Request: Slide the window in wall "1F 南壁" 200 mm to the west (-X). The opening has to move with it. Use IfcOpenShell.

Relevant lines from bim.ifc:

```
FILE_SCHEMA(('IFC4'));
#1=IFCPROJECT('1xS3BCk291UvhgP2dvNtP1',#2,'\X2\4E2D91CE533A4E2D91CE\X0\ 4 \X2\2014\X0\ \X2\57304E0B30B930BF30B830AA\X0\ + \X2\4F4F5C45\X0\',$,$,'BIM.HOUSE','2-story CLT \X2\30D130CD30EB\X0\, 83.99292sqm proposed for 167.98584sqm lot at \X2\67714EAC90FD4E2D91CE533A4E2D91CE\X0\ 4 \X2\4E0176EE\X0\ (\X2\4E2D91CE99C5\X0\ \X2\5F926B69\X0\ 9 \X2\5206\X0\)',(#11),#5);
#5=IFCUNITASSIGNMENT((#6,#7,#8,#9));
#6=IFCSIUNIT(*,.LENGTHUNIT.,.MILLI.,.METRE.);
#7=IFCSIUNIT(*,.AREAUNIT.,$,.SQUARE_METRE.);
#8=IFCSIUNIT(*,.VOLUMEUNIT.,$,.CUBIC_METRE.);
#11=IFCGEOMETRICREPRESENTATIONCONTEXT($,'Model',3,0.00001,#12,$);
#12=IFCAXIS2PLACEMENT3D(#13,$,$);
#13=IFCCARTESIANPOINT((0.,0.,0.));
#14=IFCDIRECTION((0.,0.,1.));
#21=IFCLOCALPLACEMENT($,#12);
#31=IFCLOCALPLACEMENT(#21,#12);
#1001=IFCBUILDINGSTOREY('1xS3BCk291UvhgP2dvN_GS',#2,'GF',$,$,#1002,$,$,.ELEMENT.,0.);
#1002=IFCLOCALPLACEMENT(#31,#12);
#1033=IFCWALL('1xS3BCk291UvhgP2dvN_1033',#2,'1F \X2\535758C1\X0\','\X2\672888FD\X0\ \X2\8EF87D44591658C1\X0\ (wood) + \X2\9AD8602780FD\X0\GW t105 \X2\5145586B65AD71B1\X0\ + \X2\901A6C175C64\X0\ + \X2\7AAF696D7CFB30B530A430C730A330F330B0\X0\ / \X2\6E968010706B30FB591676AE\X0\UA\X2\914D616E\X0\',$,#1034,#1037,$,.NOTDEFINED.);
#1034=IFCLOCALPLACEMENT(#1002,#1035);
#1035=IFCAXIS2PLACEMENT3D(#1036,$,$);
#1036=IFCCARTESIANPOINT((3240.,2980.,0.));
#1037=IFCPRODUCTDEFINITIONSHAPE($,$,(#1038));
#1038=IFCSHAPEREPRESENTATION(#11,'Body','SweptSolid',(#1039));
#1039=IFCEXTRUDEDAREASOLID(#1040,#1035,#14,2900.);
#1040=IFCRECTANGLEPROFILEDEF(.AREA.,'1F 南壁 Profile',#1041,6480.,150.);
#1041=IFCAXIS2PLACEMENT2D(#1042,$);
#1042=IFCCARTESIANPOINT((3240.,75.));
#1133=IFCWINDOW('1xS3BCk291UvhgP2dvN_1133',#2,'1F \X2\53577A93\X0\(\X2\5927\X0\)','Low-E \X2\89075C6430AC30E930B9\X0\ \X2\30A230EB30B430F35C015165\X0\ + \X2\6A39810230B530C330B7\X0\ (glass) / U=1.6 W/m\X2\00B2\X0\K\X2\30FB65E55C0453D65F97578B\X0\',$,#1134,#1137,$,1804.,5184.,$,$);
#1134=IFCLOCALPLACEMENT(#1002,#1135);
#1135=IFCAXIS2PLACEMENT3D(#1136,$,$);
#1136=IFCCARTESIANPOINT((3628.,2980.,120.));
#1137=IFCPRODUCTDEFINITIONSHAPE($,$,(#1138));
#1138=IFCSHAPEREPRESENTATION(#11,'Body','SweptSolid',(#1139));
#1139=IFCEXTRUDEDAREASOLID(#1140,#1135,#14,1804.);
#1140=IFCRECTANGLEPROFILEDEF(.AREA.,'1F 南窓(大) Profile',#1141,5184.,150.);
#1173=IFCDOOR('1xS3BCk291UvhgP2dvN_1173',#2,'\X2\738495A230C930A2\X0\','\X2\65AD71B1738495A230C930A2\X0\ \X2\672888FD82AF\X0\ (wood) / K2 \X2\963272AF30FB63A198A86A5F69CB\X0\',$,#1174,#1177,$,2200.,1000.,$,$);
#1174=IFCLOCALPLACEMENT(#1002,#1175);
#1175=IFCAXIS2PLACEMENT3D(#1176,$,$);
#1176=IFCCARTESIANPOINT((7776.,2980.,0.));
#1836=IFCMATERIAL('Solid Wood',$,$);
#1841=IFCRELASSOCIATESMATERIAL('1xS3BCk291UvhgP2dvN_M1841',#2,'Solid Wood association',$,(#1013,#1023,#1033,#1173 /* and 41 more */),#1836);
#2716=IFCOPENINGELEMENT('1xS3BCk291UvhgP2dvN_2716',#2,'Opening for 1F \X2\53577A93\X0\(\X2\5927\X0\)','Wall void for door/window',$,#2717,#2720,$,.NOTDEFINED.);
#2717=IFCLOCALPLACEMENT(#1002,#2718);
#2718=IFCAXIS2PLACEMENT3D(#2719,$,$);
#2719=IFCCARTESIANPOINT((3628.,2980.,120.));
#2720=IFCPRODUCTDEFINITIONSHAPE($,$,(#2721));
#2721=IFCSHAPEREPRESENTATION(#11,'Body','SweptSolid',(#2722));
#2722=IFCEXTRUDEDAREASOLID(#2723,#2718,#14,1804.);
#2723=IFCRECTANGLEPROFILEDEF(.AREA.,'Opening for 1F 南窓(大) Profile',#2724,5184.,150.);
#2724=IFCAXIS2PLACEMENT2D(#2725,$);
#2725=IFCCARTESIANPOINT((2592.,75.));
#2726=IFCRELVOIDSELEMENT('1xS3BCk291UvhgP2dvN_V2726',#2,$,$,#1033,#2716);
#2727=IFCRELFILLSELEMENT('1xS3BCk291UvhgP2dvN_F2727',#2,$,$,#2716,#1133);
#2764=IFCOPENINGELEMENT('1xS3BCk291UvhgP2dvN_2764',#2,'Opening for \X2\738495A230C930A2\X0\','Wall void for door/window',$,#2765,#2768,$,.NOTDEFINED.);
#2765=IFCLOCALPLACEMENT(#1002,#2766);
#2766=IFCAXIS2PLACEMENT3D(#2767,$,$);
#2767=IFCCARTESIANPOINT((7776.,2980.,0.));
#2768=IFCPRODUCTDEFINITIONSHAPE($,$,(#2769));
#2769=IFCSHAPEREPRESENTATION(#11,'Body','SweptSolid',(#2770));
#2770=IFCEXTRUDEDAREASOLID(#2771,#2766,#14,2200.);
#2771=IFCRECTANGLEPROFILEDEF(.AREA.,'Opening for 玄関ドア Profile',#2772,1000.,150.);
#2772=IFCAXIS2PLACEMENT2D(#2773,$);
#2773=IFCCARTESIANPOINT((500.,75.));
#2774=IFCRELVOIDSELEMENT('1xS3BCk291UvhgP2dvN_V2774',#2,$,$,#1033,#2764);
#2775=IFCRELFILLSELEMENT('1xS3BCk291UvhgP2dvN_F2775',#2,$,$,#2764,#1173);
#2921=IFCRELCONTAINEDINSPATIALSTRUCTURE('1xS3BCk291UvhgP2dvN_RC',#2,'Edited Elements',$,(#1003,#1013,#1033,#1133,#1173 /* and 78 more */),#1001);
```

```python
import ifcopenshell
import ifcopenshell.api.geometry
import ifcopenshell.util.placement
import ifcopenshell.util.unit

model = ifcopenshell.open("bim.ifc")
unit_scale = ifcopenshell.util.unit.calculate_unit_scale(model)

window = model.by_guid("1xS3BCk291UvhgP2dvN_1133")
opening = window.FillsVoids[0].RelatingOpeningElement
wall = opening.VoidsElements[0].RelatingBuildingElement

wall_matrix = ifcopenshell.util.placement.get_local_placement(wall.ObjectPlacement)
shift = wall_matrix[:3, 0] * -0.2 / unit_scale
before = ifcopenshell.util.placement.get_local_placement(window.ObjectPlacement)[:3, 3].copy()

# The window is not placed relative to its opening, so move both.
for product in (opening, window):
    matrix = ifcopenshell.util.placement.get_local_placement(product.ObjectPlacement)
    matrix[:3, 3] += shift
    ifcopenshell.api.geometry.edit_object_placement(model, product=product, matrix=matrix, is_si=False)

after = ifcopenshell.util.placement.get_local_placement(window.ObjectPlacement)[:3, 3]
print("window moved by", (after - before).round(3) + 0.0)

model.write("bim_rev.ifc")
```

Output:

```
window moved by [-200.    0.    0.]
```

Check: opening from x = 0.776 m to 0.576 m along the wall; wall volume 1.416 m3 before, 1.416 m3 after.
